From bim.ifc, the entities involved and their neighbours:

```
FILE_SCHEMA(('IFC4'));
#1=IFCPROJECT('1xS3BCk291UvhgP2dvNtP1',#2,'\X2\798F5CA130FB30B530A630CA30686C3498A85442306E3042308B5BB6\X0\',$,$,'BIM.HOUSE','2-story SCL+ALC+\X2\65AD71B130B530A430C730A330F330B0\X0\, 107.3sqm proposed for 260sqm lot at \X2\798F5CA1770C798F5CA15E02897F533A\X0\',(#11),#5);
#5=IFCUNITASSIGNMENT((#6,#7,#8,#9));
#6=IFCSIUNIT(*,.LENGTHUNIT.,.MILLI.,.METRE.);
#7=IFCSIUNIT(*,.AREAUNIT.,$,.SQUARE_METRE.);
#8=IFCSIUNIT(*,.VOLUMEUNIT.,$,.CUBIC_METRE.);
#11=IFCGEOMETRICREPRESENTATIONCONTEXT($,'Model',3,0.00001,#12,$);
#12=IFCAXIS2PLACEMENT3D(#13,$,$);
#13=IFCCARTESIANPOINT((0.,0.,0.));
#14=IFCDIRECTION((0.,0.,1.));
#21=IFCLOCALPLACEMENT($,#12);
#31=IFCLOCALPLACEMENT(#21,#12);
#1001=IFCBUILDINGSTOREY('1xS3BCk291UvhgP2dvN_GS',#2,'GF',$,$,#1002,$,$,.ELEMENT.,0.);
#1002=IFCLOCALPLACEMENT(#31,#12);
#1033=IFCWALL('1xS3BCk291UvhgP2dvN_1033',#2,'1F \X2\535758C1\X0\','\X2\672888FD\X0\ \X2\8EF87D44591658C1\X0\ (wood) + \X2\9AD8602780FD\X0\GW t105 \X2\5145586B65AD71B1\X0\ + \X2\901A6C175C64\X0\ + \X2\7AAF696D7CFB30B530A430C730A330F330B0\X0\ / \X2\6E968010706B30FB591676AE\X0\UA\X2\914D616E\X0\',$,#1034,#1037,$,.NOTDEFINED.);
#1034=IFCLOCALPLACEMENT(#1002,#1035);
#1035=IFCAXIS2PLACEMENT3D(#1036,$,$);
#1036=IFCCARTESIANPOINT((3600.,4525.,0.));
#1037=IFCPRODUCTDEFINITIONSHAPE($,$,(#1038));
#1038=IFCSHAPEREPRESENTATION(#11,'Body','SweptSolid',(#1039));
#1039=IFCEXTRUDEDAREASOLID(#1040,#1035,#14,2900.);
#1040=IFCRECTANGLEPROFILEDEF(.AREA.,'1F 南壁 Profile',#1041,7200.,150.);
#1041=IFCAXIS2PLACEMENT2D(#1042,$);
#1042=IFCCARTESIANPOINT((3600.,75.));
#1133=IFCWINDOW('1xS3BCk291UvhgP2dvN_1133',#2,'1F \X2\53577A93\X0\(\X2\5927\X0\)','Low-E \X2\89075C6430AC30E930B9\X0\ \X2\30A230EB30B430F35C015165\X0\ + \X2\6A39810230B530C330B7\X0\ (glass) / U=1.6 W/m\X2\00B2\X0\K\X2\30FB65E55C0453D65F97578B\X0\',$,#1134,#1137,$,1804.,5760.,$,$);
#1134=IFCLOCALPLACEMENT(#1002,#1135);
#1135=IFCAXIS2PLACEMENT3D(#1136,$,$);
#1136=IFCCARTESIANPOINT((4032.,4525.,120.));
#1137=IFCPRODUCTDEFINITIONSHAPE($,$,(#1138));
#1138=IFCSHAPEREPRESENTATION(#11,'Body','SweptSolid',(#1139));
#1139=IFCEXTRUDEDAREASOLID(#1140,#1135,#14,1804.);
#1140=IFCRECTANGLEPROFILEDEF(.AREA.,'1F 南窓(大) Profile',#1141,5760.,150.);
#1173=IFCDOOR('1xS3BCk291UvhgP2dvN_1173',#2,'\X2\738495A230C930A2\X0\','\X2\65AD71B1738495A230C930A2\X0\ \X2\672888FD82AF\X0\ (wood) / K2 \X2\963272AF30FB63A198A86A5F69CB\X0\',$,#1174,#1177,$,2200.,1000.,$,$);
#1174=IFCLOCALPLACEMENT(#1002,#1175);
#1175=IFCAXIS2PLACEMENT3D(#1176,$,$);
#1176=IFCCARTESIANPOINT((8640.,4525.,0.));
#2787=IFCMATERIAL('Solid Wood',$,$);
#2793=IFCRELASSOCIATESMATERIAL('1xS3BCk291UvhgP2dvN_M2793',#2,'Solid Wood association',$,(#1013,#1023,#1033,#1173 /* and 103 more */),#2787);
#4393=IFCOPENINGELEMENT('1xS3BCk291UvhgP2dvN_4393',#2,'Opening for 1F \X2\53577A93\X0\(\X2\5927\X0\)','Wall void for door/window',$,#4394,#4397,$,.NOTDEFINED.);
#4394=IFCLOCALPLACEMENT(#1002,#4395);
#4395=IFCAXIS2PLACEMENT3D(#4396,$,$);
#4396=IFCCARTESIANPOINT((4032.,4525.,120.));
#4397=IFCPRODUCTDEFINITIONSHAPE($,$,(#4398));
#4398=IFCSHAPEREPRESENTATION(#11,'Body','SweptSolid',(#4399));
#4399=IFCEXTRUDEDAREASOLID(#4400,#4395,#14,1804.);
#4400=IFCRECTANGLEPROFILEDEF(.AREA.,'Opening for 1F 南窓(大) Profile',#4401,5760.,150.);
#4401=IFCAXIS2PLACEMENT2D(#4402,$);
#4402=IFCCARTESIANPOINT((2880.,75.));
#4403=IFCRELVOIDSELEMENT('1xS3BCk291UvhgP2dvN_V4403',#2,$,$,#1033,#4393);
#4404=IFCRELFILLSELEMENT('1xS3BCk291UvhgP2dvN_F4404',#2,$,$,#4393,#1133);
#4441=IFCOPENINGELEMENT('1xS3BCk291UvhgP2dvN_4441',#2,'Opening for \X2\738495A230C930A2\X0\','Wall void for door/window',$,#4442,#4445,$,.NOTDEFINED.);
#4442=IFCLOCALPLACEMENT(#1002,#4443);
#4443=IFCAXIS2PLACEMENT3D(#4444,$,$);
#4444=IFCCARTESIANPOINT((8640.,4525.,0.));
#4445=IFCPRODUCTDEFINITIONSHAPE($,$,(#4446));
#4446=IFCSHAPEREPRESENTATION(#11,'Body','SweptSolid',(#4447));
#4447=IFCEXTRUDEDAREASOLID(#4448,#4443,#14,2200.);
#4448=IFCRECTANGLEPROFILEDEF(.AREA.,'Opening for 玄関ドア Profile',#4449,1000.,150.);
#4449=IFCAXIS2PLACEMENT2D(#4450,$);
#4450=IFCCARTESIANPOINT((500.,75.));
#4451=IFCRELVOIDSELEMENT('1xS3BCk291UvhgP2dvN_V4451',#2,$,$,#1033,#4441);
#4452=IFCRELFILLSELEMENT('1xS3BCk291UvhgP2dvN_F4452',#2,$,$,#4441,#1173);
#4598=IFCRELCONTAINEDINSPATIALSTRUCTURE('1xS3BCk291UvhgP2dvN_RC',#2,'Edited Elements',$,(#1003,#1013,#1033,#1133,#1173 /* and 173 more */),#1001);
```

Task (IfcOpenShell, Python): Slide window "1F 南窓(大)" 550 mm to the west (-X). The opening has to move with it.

```python
import ifcopenshell
import ifcopenshell.api.geometry
import ifcopenshell.util.placement
import ifcopenshell.util.unit

model = ifcopenshell.open("bim.ifc")
unit_scale = ifcopenshell.util.unit.calculate_unit_scale(model)

window = model.by_guid("1xS3BCk291UvhgP2dvN_1133")
opening = window.FillsVoids[0].RelatingOpeningElement
wall = opening.VoidsElements[0].RelatingBuildingElement

wall_matrix = ifcopenshell.util.placement.get_local_placement(wall.ObjectPlacement)
shift = wall_matrix[:3, 0] * -0.55 / unit_scale
before = ifcopenshell.util.placement.get_local_placement(window.ObjectPlacement)[:3, 3].copy()

# The window is not placed relative to its opening, so move both.
for product in (opening, window):
    matrix = ifcopenshell.util.placement.get_local_placement(product.ObjectPlacement)
    matrix[:3, 3] += shift
    ifcopenshell.api.geometry.edit_object_placement(model, product=product, matrix=matrix, is_si=False)

after = ifcopenshell.util.placement.get_local_placement(window.ObjectPlacement)[:3, 3]
print("window moved by", (after - before).round(3) + 0.0)

model.write("bim-out.ifc")
```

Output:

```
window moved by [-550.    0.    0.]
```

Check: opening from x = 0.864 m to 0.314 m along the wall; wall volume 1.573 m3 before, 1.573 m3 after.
